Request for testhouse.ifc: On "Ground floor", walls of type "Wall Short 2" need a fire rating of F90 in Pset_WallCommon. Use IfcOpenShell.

First a look at what the model holds.

```python
import ifcopenshell
import ifcopenshell.util.element

model = ifcopenshell.open("testhouse.ifc")
print(model.schema)
storey = next(s for s in model.by_type("IfcBuildingStorey") if s.Name == "Ground floor")
walls = [e for e in ifcopenshell.util.element.get_decomposition(storey) if e.is_a("IfcWall")]
seen = {}
for e in walls:
    element_type = ifcopenshell.util.element.get_type(e)
    key = (element_type.Name if element_type != e and element_type else None, ifcopenshell.util.element.get_pset(e, "Pset_WallCommon", "FireRating"))
    seen[key] = seen.get(key, 0) + 1
for (name, value), count in sorted(seen.items(), key=str):
    print(count, "x", name, "|", value)
```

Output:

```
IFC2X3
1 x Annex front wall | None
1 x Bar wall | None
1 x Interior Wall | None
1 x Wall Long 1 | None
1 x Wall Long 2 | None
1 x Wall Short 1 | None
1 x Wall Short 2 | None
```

```python
import ifcopenshell
import ifcopenshell.api.pset
import ifcopenshell.util.element

model = ifcopenshell.open("testhouse.ifc")

storey = next(s for s in model.by_type("IfcBuildingStorey") if s.Name == "Ground floor")
walls = [e for e in ifcopenshell.util.element.get_decomposition(storey) if e.is_a("IfcWall")]

count = 0
for e in walls:
    element_type = ifcopenshell.util.element.get_type(e)
    if element_type in (None, e) or element_type.Name != "Wall Short 2":
        continue
    # add_pset returns the element's existing set when there is one.
    pset = ifcopenshell.api.pset.add_pset(model, product=e, name="Pset_WallCommon")
    ifcopenshell.api.pset.edit_pset(model, pset=pset, properties={"FireRating": "F90"})
    count += 1

print(count, "walls updated")

model.write("testhouse_edited.ifc")
```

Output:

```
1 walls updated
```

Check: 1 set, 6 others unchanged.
